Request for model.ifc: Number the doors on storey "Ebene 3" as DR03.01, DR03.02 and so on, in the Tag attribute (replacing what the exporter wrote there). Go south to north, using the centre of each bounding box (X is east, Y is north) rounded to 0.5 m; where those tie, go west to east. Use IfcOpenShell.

First a look at what the model holds.

```python
import ifcopenshell
import ifcopenshell.util.element
import ifcopenshell.util.placement

model = ifcopenshell.open("model.ifc")
print(model.schema)
storey = next(s for s in model.by_type("IfcBuildingStorey") if s.Name == "Ebene 3")
doors = [e for e in ifcopenshell.util.element.get_decomposition(storey) if e.is_a("IfcDoor")]
for e in sorted(doors, key=lambda e: e.id()):
    origin = ifcopenshell.util.placement.get_local_placement(e.ObjectPlacement)[:3, 3]
    print(e.id(), e.Tag, e.Name, origin.round(2) + 0.0, sep=" | ")
```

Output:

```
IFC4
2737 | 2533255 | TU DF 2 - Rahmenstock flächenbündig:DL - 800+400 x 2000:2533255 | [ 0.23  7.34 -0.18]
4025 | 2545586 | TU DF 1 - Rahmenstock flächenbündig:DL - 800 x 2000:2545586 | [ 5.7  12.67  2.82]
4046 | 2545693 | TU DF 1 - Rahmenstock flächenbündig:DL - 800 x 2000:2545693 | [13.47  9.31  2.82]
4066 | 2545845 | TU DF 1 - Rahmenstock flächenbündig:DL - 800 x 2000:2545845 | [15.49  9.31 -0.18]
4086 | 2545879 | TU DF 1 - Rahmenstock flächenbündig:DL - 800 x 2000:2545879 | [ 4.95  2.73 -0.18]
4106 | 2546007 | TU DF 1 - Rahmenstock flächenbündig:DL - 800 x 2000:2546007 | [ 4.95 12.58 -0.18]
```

```python
import ifcopenshell
import ifcopenshell.geom
import ifcopenshell.util.element
import ifcopenshell.util.shape

model = ifcopenshell.open("model.ifc")
settings = ifcopenshell.geom.settings()
settings.set("use-world-coords", True)


def centre(element):
    shape = ifcopenshell.geom.create_shape(settings, element)
    return ifcopenshell.util.shape.get_bbox_centroid(shape.geometry)


storey = next(s for s in model.by_type("IfcBuildingStorey") if s.Name == "Ebene 3")
doors = [e for e in ifcopenshell.util.element.get_decomposition(storey) if e.is_a("IfcDoor")]

# Insertion points can sit at a corner or the storey origin, so sort by the geometry (in metres).
centres = {e: centre(e) for e in doors}
doors.sort(key=lambda e: (round(centres[e][1] / 0.5), centres[e][0]))

for i, e in enumerate(doors, start=1):
    number = f"DR03.{i:02d}"
    e.Tag = number
    print(e.id(), number)

model.write("model_updated.ifc")
```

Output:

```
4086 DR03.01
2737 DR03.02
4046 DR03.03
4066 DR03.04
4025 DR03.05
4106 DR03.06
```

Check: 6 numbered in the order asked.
